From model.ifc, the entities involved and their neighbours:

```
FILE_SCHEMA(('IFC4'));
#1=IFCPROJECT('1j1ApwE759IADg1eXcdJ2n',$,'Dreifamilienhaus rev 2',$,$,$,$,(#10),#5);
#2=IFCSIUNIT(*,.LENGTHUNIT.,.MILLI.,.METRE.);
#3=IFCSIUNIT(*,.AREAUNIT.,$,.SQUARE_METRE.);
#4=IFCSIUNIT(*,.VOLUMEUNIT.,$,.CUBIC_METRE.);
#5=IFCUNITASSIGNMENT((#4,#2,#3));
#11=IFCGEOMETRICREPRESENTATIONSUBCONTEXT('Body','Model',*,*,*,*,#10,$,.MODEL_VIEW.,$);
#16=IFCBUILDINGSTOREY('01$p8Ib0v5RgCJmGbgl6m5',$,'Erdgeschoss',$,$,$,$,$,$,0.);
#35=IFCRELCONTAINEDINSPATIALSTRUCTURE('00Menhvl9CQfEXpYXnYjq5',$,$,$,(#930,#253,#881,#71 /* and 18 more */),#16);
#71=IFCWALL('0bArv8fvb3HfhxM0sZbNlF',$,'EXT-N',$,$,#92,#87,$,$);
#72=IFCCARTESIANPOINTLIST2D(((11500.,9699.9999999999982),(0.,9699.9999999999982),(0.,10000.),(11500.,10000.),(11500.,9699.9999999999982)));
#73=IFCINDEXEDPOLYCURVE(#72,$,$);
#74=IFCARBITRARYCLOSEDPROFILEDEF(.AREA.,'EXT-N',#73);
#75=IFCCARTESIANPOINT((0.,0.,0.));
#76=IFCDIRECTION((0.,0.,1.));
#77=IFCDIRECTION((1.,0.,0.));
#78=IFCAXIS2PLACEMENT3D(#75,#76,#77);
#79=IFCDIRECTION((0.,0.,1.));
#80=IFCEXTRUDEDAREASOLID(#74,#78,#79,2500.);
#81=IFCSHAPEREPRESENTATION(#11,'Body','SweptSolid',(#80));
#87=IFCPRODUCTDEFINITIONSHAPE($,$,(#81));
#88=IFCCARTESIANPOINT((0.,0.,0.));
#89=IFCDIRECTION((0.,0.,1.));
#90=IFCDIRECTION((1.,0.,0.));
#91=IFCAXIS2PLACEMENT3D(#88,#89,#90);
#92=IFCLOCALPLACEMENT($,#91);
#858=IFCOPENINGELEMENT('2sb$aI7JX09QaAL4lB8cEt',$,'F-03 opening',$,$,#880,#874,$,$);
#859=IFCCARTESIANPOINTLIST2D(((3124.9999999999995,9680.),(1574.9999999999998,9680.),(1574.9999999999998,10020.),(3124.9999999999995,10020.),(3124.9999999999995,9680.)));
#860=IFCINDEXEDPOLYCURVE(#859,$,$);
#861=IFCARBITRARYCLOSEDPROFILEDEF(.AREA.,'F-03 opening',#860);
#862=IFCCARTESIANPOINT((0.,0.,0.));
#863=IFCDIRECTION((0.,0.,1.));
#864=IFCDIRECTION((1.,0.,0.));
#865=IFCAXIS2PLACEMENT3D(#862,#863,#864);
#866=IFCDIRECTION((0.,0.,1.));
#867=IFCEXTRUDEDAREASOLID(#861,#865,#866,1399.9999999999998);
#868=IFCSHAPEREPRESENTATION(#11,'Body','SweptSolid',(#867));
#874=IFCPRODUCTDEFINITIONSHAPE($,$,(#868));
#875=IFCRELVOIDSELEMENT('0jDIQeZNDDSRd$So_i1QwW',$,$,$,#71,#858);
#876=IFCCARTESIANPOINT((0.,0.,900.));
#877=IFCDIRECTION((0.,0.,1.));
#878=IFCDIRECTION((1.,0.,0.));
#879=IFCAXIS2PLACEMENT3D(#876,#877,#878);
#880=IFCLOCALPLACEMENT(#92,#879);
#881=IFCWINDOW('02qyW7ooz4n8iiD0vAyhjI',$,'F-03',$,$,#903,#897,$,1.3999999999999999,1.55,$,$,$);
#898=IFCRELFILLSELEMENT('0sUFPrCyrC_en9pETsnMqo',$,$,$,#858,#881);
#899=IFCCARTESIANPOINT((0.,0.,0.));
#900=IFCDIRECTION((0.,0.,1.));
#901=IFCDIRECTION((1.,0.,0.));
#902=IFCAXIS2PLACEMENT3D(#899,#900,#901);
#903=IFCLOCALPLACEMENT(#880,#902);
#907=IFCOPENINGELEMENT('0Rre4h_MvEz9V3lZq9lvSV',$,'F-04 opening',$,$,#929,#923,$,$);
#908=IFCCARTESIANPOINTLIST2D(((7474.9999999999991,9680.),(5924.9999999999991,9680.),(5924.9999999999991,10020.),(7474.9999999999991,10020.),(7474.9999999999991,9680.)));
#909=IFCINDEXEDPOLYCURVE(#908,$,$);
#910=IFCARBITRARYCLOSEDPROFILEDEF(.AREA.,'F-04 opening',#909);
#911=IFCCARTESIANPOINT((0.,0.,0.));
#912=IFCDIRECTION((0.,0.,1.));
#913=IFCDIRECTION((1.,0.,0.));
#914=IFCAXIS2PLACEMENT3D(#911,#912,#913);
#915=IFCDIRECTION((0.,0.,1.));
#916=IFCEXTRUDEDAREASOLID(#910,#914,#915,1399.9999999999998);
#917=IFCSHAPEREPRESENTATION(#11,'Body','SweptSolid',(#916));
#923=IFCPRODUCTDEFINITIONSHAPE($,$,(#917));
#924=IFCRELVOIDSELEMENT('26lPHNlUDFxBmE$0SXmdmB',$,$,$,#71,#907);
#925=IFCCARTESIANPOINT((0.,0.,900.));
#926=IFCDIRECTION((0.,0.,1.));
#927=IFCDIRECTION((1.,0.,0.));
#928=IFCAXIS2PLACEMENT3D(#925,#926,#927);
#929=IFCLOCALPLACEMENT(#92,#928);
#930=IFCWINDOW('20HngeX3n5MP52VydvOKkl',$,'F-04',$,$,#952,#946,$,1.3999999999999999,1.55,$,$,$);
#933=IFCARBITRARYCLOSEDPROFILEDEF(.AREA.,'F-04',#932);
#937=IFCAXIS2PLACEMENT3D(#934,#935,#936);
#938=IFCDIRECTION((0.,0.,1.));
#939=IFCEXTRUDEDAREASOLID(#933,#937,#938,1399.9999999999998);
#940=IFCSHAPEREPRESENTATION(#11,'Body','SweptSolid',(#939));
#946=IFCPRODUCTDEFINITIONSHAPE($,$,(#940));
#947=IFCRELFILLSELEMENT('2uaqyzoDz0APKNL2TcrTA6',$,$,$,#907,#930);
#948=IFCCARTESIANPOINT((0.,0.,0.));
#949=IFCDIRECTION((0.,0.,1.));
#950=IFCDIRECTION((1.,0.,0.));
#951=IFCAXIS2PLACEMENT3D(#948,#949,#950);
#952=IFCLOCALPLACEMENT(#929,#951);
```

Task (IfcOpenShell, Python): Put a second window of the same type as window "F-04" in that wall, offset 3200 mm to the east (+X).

```python
import ifcopenshell
import ifcopenshell.api.feature
import ifcopenshell.api.geometry
import ifcopenshell.api.root
import ifcopenshell.geom
import ifcopenshell.util.element
import ifcopenshell.util.placement
import ifcopenshell.util.shape
import ifcopenshell.util.unit

model = ifcopenshell.open("model.ifc")
unit_scale = ifcopenshell.util.unit.calculate_unit_scale(model)
settings = ifcopenshell.geom.settings()


def volume(element):
    """Net volume in cubic metres, openings subtracted."""
    shape = ifcopenshell.geom.create_shape(settings, element)
    return ifcopenshell.util.shape.get_volume(shape.geometry)


window = model.by_guid("20HngeX3n5MP52VydvOKkl")
opening = window.FillsVoids[0].RelatingOpeningElement
wall = opening.VoidsElements[0].RelatingBuildingElement
before = volume(wall)
shift = ifcopenshell.util.placement.get_local_placement(wall.ObjectPlacement)[:3, 0] * 3.2 / unit_scale

# copy_class copies the void relationship, type, container and properties, but no geometry.
new_opening = ifcopenshell.api.root.copy_class(model, product=opening)
new_opening.Representation = ifcopenshell.util.element.copy_deep(
    model, opening.Representation, exclude=["IfcGeometricRepresentationContext", "IfcRepresentationMap"]
)
new_window = ifcopenshell.api.root.copy_class(model, product=window)
new_window.Representation = ifcopenshell.util.element.copy_deep(
    model, window.Representation, exclude=["IfcGeometricRepresentationContext", "IfcRepresentationMap"]
)
ifcopenshell.api.feature.add_filling(model, opening=new_opening, element=new_window)

for old, new in ((opening, new_opening), (window, new_window)):
    matrix = ifcopenshell.util.placement.get_local_placement(old.ObjectPlacement)
    matrix[:3, 3] += shift
    ifcopenshell.api.geometry.edit_object_placement(model, product=new, matrix=matrix, is_si=False)

after = volume(wall)

print(f"wall volume {before:.3f} -> {after:.3f} m3")

model.write("model_edited.ifc")
```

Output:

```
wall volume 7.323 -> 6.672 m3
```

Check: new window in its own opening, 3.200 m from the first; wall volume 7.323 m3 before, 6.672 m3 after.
